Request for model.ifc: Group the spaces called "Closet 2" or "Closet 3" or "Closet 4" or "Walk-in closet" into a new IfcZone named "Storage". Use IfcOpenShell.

First a look at what the model holds.

```python
import ifcopenshell

model = ifcopenshell.open("model.ifc")
print(model.schema)
seen = {}
for space in model.by_type("IfcSpace"):
    seen[space.LongName] = seen.get(space.LongName, 0) + 1
for name, count in sorted(seen.items(), key=str):
    print(count, "x", name)
print("zones:", [z.Name for z in model.by_type("IfcZone")][:20])
```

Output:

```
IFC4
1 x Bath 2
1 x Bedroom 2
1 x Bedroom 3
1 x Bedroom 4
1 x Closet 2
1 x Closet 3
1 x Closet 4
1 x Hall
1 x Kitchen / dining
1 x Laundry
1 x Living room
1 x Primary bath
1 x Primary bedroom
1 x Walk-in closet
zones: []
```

```python
import ifcopenshell
import ifcopenshell.api.group
import ifcopenshell.api.root

model = ifcopenshell.open("model.ifc")

names = {"Closet 2", "Closet 3", "Closet 4", "Walk-in closet"}
spaces = [s for s in model.by_type("IfcSpace") if s.LongName in names]

zone = ifcopenshell.api.root.create_entity(model, ifc_class="IfcZone", name="Storage")
ifcopenshell.api.group.assign_group(model, products=spaces, group=zone)
print(len(spaces), "spaces in", zone.Name)

model.write("model_edited.ifc")
```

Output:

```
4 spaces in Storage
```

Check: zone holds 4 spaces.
